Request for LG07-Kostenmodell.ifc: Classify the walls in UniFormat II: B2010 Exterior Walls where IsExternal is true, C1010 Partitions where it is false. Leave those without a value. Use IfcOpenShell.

First a look at what the model holds.

```python
import ifcopenshell
import ifcopenshell.util.element

model = ifcopenshell.open("LG07-Kostenmodell.ifc")
print(model.schema)
print("classifications:", [c.Name for c in model.by_type("IfcClassification")])
values = [ifcopenshell.util.element.get_pset(e, "Pset_WallCommon", "IsExternal") for e in model.by_type("IfcWall")]
for value in (True, False, None):
    print("IsExternal", value, values.count(value))
```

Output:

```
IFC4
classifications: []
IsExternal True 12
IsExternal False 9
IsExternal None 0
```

```python
import ifcopenshell
import ifcopenshell.api.classification
import ifcopenshell.util.element

model = ifcopenshell.open("LG07-Kostenmodell.ifc")

system = ifcopenshell.api.classification.add_classification(model, classification="UniFormat II")

walls = model.by_type("IfcWall")
external = {e: ifcopenshell.util.element.get_pset(e, "Pset_WallCommon", "IsExternal") for e in walls}
for flag, code, name in ((True, "B2010", "Exterior Walls"), (False, "C1010", "Partitions")):
    products = [e for e in walls if external[e] is flag]
    ifcopenshell.api.classification.add_reference(
        model, products=products, classification=system, identification=code, name=name
    )
    print(code, len(products))

model.write("LG07-Kostenmodell_v2.ifc")
```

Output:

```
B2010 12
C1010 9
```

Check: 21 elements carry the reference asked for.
